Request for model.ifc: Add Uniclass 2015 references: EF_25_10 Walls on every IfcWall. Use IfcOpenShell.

First a look at what the model holds.

```python
import ifcopenshell

model = ifcopenshell.open("model.ifc")
print(model.schema)
print("classifications:", [c.Name for c in model.by_type("IfcClassification")])
for ifc_class in ("IfcDoor", "IfcRoof", "IfcStair", "IfcWall", "IfcWindow"):
    print(ifc_class, len(model.by_type(ifc_class)))
```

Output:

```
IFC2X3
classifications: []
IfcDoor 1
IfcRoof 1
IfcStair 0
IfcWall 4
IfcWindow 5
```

```python
import ifcopenshell
import ifcopenshell.api.classification

model = ifcopenshell.open("model.ifc")

# IFC2X3 requires Source and Edition and has no link from the project to the system.
system = model.create_entity("IfcClassification", Source="NBS", Edition="2015", Name="Uniclass 2015")

codes = {
    "IfcWall": ("EF_25_10", "Walls"),
}
for ifc_class, (code, name) in codes.items():
    products = model.by_type(ifc_class)
    ifcopenshell.api.classification.add_reference(
        model, products=products, classification=system, identification=code, name=name
    )
    print(code, len(products))

model.write("model_rev.ifc")
```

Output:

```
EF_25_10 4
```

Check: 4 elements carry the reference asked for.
